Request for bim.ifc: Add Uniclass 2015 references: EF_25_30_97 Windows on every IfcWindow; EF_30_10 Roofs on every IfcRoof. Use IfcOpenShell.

First a look at what the model holds.

```python
import ifcopenshell

model = ifcopenshell.open("bim.ifc")
print(model.schema)
print("classifications:", [c.Name for c in model.by_type("IfcClassification")])
for ifc_class in ("IfcDoor", "IfcRoof", "IfcStair", "IfcWall", "IfcWindow"):
    print(ifc_class, len(model.by_type(ifc_class)))
```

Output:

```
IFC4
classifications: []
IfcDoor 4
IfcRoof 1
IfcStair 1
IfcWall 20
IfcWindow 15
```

```python
import ifcopenshell
import ifcopenshell.api.classification

model = ifcopenshell.open("bim.ifc")

system = ifcopenshell.api.classification.add_classification(model, classification="Uniclass 2015")

codes = {
    "IfcWindow": ("EF_25_30_97", "Windows"),
    "IfcRoof": ("EF_30_10", "Roofs"),
}
for ifc_class, (code, name) in codes.items():
    products = model.by_type(ifc_class)
    ifcopenshell.api.classification.add_reference(
        model, products=products, classification=system, identification=code, name=name
    )
    print(code, len(products))

model.write("bim-out.ifc")
```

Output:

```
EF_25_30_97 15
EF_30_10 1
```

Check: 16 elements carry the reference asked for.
